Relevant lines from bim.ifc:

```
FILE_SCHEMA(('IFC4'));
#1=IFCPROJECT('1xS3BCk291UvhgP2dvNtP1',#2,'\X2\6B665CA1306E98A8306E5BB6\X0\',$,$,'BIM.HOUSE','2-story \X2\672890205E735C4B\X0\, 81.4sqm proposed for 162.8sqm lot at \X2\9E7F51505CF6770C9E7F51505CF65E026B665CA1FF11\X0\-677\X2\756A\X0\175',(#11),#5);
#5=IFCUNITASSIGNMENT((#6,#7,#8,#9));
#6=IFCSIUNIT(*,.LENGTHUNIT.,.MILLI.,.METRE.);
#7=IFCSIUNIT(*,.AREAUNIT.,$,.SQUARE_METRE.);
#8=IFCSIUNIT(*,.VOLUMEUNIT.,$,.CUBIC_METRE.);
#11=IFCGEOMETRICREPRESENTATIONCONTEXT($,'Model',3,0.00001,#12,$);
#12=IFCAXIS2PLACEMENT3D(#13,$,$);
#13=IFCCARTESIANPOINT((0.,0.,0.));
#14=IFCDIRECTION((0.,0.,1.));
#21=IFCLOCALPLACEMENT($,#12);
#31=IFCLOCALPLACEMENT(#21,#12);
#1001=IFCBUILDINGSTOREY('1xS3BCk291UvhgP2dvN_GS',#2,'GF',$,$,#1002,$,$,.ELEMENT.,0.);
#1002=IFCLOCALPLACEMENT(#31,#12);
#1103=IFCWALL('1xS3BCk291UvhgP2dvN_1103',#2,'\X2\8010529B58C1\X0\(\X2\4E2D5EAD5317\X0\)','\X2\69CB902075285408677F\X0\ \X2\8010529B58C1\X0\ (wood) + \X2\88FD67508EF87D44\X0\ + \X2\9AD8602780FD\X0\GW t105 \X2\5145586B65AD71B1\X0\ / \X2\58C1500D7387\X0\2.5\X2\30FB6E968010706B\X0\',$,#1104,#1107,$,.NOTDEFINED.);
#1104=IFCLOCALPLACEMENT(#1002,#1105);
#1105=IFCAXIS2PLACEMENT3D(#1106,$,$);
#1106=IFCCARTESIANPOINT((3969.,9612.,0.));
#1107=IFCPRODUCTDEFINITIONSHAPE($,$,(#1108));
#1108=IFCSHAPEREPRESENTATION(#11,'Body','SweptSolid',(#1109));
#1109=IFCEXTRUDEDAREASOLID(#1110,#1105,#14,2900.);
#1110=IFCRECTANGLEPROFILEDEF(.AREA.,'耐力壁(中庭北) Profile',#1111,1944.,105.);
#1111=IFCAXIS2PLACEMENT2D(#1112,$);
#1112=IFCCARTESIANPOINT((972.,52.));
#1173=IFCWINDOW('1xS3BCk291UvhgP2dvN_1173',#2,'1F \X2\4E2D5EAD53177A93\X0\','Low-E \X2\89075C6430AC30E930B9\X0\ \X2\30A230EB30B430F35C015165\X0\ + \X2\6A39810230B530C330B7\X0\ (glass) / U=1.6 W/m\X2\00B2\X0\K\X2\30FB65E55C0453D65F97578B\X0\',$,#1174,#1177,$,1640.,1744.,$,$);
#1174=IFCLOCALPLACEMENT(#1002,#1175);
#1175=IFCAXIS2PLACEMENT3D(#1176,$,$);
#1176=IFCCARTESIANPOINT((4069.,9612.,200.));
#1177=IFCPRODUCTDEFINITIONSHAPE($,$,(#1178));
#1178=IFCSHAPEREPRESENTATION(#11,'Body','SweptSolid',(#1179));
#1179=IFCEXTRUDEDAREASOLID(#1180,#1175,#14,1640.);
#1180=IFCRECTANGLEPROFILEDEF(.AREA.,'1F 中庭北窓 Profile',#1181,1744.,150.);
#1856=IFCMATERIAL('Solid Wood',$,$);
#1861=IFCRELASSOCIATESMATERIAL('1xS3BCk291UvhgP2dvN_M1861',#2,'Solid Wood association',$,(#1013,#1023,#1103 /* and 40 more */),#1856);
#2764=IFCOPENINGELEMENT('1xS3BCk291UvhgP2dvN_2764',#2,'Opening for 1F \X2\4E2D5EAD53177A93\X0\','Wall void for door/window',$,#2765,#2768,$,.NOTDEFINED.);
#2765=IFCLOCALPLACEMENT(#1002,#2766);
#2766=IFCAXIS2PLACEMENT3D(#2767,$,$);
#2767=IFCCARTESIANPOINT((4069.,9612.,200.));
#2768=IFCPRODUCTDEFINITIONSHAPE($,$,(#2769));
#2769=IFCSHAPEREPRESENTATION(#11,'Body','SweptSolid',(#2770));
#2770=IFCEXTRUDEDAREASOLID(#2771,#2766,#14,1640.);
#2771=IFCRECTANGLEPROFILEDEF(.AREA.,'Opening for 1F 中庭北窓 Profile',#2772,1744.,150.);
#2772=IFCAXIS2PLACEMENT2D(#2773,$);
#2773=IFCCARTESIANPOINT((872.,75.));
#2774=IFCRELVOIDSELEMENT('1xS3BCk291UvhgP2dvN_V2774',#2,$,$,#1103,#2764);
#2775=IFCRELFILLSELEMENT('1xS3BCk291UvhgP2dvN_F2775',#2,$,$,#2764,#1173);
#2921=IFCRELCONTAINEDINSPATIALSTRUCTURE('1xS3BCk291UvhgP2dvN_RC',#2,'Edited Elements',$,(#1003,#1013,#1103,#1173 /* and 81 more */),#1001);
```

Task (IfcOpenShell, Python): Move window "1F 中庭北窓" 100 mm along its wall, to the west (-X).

```python
import ifcopenshell
import ifcopenshell.api.geometry
import ifcopenshell.util.placement

model = ifcopenshell.open("bim.ifc")

window = model.by_guid("1xS3BCk291UvhgP2dvN_1173")
opening = window.FillsVoids[0].RelatingOpeningElement
wall = opening.VoidsElements[0].RelatingBuildingElement

wall_matrix = ifcopenshell.util.placement.get_local_placement(wall.ObjectPlacement)
shift = wall_matrix[:3, 0] * -100.0
before = ifcopenshell.util.placement.get_local_placement(window.ObjectPlacement)[:3, 3].copy()

# The window is not placed relative to its opening, so move both.
for product in (opening, window):
    matrix = ifcopenshell.util.placement.get_local_placement(product.ObjectPlacement)
    matrix[:3, 3] += shift
    ifcopenshell.api.geometry.edit_object_placement(model, product=product, matrix=matrix, is_si=False)

after = ifcopenshell.util.placement.get_local_placement(window.ObjectPlacement)[:3, 3]
print("window moved by", (after - before).round(3) + 0.0)

model.write("bim_rev.ifc")
```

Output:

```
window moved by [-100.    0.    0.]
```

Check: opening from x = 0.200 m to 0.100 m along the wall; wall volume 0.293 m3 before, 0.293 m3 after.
